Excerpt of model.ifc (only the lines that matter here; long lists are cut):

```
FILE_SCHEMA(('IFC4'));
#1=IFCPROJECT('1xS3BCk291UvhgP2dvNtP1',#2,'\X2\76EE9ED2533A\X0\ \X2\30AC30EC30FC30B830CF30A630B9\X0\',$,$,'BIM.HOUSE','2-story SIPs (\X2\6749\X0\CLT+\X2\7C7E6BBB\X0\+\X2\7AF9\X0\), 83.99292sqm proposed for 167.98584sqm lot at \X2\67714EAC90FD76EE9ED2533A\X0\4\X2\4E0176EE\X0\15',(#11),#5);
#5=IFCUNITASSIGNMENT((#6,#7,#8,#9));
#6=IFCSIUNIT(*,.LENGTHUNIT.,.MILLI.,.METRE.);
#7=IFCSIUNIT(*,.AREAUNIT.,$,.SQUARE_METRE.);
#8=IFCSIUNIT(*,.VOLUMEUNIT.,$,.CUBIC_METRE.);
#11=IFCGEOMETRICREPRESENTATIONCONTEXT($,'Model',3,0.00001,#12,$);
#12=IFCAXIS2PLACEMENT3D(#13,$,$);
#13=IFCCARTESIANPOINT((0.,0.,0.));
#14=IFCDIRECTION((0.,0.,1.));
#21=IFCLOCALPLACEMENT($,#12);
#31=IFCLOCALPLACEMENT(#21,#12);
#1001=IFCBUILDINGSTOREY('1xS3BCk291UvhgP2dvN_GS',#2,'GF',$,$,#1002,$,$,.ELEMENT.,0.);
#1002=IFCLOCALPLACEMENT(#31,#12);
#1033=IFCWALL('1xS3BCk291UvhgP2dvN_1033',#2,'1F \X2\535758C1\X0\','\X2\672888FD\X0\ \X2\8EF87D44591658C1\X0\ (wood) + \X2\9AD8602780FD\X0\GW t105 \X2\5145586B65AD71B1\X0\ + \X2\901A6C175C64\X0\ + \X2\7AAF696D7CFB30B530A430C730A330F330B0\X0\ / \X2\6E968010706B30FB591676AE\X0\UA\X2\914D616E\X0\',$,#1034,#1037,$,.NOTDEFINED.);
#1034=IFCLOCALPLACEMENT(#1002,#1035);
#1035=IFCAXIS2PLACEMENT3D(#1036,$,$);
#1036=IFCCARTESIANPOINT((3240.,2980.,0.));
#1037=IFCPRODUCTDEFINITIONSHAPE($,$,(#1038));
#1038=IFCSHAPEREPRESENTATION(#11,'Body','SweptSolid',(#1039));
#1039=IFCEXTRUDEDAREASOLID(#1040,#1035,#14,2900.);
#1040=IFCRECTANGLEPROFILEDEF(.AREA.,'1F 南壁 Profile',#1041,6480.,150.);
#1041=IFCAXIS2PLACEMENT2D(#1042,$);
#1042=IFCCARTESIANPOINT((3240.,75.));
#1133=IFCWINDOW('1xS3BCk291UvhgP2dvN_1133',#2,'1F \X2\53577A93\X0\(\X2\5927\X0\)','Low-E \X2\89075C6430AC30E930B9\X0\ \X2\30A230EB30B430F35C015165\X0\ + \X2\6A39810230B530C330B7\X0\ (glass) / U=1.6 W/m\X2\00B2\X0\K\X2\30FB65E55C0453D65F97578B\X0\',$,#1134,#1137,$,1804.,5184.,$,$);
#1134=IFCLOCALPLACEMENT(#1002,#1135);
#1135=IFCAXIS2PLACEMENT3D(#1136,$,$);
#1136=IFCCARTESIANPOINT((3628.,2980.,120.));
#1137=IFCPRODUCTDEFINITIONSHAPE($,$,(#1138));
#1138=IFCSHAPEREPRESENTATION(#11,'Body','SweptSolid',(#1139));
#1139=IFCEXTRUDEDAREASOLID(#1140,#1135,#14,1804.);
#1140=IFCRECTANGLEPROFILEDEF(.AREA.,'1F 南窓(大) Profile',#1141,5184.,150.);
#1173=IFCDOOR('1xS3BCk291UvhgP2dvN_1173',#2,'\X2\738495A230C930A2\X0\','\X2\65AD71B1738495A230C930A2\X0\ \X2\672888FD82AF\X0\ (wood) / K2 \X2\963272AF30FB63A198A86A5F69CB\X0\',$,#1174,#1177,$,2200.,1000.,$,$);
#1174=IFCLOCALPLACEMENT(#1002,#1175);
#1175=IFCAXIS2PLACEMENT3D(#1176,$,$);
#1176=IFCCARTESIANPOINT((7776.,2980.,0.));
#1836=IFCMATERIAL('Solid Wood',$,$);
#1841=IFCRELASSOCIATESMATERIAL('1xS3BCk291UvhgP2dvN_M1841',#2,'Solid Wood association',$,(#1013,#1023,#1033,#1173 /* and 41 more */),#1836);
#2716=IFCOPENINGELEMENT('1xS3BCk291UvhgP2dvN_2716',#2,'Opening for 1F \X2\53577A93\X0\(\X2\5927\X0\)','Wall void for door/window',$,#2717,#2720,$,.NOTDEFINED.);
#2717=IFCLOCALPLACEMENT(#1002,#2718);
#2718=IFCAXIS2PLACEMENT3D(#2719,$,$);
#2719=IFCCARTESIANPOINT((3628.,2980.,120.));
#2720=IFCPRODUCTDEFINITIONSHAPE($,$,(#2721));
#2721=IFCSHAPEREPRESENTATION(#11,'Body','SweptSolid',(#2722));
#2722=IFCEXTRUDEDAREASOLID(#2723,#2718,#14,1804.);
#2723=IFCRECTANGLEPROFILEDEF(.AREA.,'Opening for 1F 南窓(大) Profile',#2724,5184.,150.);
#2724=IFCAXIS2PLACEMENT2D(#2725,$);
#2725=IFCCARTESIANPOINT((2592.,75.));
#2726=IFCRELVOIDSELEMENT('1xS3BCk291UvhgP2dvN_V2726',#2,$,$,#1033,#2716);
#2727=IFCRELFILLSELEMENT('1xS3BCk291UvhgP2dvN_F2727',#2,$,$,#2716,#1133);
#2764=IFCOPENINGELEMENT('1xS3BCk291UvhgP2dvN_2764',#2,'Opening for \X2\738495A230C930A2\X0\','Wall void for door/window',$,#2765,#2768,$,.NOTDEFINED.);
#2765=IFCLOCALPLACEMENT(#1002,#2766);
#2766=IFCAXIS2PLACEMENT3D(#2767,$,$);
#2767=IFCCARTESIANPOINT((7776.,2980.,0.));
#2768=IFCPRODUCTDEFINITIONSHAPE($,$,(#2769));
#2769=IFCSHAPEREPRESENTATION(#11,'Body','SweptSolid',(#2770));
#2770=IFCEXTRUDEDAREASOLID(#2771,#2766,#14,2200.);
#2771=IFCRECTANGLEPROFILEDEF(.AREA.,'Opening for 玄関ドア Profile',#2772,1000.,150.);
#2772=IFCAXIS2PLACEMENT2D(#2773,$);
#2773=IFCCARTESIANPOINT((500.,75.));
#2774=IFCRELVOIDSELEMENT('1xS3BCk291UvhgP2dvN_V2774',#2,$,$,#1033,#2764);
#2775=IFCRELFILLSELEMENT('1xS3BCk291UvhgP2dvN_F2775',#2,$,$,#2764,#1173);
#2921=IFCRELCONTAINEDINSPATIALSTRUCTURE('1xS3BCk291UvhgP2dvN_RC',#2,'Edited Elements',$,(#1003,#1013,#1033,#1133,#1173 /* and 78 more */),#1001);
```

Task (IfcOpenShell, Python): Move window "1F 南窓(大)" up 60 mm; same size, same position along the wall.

```python
import numpy as np
import ifcopenshell
import ifcopenshell.api.geometry
import ifcopenshell.util.placement
import ifcopenshell.util.unit

model = ifcopenshell.open("model.ifc")
unit_scale = ifcopenshell.util.unit.calculate_unit_scale(model)

window = model.by_guid("1xS3BCk291UvhgP2dvN_1133")
opening = window.FillsVoids[0].RelatingOpeningElement
dz = 0.06 / unit_scale

shift = np.array([0.0, 0.0, dz])
# The window is not placed relative to its opening, so move both.
for product in (opening, window):
    matrix = ifcopenshell.util.placement.get_local_placement(product.ObjectPlacement)
    matrix[:3, 3] += shift
    ifcopenshell.api.geometry.edit_object_placement(model, product=product, matrix=matrix, is_si=False)

print(f"moved by {dz * unit_scale:+.3f} m")

model.write("model_updated.ifc")
```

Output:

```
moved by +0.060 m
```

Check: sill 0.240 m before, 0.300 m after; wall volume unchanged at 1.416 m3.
